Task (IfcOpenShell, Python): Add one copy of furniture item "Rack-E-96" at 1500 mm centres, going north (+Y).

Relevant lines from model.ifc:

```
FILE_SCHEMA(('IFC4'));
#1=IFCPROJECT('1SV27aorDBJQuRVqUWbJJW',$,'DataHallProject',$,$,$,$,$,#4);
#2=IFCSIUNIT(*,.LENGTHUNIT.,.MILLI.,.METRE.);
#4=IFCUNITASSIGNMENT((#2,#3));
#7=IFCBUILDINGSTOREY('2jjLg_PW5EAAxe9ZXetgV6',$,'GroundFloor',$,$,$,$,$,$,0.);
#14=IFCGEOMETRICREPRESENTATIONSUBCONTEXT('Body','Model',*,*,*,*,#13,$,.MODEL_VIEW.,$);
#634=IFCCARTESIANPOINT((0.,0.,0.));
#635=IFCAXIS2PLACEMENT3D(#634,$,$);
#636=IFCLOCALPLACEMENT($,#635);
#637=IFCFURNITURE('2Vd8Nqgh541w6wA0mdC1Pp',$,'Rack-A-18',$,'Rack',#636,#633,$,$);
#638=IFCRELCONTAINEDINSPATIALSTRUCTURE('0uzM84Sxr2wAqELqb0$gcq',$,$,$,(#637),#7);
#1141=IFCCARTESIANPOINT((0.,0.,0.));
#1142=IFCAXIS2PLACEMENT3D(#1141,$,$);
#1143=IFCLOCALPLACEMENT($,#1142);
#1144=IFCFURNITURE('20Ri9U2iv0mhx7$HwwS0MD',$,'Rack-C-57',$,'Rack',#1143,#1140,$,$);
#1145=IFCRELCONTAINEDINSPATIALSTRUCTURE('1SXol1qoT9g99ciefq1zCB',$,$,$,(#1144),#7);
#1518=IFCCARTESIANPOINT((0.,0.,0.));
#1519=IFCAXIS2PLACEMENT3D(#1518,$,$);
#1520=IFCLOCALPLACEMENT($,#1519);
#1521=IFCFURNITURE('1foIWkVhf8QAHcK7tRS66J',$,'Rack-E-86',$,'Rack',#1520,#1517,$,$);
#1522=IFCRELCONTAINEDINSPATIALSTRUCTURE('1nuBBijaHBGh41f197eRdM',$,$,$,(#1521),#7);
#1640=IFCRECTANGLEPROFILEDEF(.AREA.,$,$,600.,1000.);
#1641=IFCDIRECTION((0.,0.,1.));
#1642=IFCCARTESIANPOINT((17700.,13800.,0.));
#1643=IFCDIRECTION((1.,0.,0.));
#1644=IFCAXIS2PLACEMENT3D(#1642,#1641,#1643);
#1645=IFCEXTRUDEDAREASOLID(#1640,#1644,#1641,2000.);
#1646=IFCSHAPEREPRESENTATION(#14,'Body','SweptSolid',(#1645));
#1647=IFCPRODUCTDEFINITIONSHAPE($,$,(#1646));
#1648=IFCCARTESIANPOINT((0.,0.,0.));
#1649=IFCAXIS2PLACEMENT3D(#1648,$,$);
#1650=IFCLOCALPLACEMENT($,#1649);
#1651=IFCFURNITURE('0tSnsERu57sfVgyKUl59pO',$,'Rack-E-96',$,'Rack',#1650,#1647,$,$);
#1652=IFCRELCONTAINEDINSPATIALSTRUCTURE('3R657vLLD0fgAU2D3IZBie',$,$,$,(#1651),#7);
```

```python
import numpy as np
import ifcopenshell
import ifcopenshell.api.geometry
import ifcopenshell.api.root
import ifcopenshell.util.element
import ifcopenshell.util.placement
import ifcopenshell.util.unit

model = ifcopenshell.open("model.ifc")
unit_scale = ifcopenshell.util.unit.calculate_unit_scale(model)

source = model.by_guid("0tSnsERu57sfVgyKUl59pO")
base = ifcopenshell.util.placement.get_local_placement(source.ObjectPlacement)
step = np.array([0.0, 1.0, 0.0]) * 1.5 / unit_scale

for i in range(1, 2):
    copy = ifcopenshell.api.root.copy_class(model, product=source)
    copy.Representation = ifcopenshell.util.element.copy_deep(
        model, source.Representation, exclude=["IfcGeometricRepresentationContext", "IfcRepresentationMap"]
    )
    matrix = base.copy()
    matrix[:3, 3] += i * step
    print("added at", matrix[:3, 3].round(3) + 0.0)
    ifcopenshell.api.geometry.edit_object_placement(model, product=copy, matrix=matrix, is_si=False)

model.write("model_edited.ifc")
```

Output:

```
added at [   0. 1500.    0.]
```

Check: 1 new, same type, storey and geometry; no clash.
